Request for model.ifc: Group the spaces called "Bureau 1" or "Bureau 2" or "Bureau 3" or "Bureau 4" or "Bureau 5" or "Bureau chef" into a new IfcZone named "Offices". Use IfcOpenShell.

First a look at what the model holds.

```python
import ifcopenshell

model = ifcopenshell.open("model.ifc")
print(model.schema)
seen = {}
for space in model.by_type("IfcSpace"):
    seen[space.LongName] = seen.get(space.LongName, 0) + 1
for name, count in sorted(seen.items(), key=str):
    print(count, "x", name)
print("zones:", [z.Name for z in model.by_type("IfcZone")][:20])
```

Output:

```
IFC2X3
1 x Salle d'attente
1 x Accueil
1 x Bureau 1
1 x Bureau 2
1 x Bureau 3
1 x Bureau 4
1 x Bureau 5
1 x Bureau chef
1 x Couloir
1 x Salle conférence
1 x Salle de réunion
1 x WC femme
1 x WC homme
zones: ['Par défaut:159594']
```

```python
import ifcopenshell
import ifcopenshell.api.group
import ifcopenshell.api.root

model = ifcopenshell.open("model.ifc")

names = {"Bureau 1", "Bureau 2", "Bureau 3", "Bureau 4", "Bureau 5", "Bureau chef"}
spaces = [s for s in model.by_type("IfcSpace") if s.LongName in names]

zone = ifcopenshell.api.root.create_entity(model, ifc_class="IfcZone", name="Offices")
ifcopenshell.api.group.assign_group(model, products=spaces, group=zone)
print(len(spaces), "spaces in", zone.Name)

model.write("model_edited.ifc")
```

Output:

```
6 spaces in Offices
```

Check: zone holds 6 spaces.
